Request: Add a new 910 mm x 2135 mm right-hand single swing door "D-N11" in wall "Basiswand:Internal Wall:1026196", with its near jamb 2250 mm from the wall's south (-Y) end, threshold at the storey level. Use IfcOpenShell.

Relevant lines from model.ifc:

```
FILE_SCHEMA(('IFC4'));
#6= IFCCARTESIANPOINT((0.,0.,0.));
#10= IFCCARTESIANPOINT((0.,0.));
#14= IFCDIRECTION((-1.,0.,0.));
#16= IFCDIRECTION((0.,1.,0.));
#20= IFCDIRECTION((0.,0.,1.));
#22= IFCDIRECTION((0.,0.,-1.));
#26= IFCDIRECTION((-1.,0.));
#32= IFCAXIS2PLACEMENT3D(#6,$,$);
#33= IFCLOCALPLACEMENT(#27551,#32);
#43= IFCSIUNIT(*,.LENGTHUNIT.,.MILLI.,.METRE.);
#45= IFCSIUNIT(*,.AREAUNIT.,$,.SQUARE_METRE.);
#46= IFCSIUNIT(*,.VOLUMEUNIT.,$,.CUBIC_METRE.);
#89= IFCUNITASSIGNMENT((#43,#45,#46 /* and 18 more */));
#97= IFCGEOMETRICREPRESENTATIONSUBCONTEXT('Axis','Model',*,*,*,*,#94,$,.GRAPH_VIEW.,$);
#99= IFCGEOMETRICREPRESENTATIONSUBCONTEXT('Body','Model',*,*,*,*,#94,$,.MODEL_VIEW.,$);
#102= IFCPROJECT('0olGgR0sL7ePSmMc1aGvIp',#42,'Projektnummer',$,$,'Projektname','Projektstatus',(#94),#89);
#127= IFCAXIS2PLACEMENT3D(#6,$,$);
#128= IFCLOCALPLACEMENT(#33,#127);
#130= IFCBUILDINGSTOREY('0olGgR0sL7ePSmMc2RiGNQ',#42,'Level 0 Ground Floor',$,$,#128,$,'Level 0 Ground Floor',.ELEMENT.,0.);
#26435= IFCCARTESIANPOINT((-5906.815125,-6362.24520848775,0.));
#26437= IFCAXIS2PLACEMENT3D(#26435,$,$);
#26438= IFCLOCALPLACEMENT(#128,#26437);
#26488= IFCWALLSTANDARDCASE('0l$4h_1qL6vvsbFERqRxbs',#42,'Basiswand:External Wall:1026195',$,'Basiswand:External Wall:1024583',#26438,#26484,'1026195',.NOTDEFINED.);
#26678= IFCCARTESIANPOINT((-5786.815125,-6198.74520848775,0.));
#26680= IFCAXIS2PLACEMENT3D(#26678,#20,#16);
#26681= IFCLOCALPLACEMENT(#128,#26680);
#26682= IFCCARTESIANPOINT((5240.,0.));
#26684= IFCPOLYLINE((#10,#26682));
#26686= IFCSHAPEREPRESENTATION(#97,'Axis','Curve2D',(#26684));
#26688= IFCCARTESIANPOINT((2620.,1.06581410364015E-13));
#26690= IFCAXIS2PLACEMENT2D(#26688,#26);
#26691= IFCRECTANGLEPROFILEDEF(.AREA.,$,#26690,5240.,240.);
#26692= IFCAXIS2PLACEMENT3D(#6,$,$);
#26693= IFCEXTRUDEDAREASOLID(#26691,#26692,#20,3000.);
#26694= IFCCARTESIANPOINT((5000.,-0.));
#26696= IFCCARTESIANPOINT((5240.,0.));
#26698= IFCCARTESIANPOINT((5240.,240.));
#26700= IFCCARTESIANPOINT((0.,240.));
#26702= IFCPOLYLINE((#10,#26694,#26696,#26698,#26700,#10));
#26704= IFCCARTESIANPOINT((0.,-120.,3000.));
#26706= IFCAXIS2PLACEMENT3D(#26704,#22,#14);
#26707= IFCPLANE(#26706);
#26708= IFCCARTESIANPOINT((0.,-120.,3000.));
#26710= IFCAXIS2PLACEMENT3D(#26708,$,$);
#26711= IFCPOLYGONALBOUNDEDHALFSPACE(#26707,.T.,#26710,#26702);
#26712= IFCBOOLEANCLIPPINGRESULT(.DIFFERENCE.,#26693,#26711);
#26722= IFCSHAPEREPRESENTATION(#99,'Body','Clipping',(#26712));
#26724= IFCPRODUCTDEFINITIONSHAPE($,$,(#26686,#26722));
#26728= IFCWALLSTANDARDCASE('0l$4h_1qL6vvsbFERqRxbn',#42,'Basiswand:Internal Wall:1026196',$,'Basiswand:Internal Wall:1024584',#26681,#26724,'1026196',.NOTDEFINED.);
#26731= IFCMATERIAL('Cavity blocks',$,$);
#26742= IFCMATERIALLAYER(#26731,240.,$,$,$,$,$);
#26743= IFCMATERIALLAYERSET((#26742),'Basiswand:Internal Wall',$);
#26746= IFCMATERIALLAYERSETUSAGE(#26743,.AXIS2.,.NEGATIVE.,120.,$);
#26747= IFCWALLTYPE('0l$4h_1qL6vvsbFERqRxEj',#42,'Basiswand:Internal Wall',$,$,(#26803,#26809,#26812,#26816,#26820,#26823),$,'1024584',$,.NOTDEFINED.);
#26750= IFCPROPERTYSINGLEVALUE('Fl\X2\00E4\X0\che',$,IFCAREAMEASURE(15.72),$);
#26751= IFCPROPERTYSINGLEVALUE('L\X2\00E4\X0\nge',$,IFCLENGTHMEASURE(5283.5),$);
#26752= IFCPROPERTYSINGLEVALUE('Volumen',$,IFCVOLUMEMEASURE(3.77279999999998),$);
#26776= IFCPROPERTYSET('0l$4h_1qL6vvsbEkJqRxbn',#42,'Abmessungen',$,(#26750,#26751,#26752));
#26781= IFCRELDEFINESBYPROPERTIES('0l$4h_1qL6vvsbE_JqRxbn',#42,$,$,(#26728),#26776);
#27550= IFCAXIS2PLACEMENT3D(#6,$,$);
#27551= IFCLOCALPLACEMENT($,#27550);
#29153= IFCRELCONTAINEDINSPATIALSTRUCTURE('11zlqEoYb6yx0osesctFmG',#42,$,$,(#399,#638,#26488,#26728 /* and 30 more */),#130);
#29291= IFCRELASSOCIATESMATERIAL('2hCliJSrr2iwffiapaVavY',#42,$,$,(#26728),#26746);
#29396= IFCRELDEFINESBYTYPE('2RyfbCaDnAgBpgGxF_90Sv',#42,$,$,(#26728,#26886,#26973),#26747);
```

```python
import numpy as np
import ifcopenshell
import ifcopenshell.api.feature
import ifcopenshell.api.geometry
import ifcopenshell.api.pset
import ifcopenshell.api.root
import ifcopenshell.api.spatial
import ifcopenshell.geom
import ifcopenshell.util.element
import ifcopenshell.util.placement
import ifcopenshell.util.representation
import ifcopenshell.util.shape
import ifcopenshell.util.unit

model = ifcopenshell.open("model.ifc")
unit_scale = ifcopenshell.util.unit.calculate_unit_scale(model)
area_scale = ifcopenshell.util.unit.calculate_unit_scale(model, "AREAUNIT")
volume_scale = ifcopenshell.util.unit.calculate_unit_scale(model, "VOLUMEUNIT")
settings = ifcopenshell.geom.settings()


def volume(element):
    """Net volume in cubic metres, openings subtracted."""
    shape = ifcopenshell.geom.create_shape(settings, element)
    return ifcopenshell.util.shape.get_volume(shape.geometry)


wall = model.by_id(26728)
storey = ifcopenshell.util.element.get_container(wall, ifc_class="IfcBuildingStorey")
context = ifcopenshell.util.representation.get_context(model, "Model", "Body", "MODEL_VIEW")
before = volume(wall)

width, height, from_end, sill = 0.91, 2.135, 2.25, 0.0  # metres

# The wall runs along its own X axis, and the end named is its -X end.
wall_shape = ifcopenshell.geom.create_shape(settings, wall)
x, y, z = ifcopenshell.util.shape.get_vertices(wall_shape.geometry).T
start = x.min() + from_end
face, thickness = float(y.min()), float(y.max() - y.min())
wall_matrix = ifcopenshell.util.placement.get_local_placement(wall.ObjectPlacement)
level = ifcopenshell.util.placement.get_local_placement(storey.ObjectPlacement)[2, 3]


def in_wall(x, y):
    """Placement at x, y metres in the wall's axes, at sill height."""
    matrix = wall_matrix.copy()
    matrix[:, 3] = wall_matrix @ np.array([x / unit_scale, y / unit_scale, 0.0, 1.0])
    matrix[2, 3] = level + sill / unit_scale
    return matrix


# Opening: a box that overshoots both wall faces by 50 mm.
opening = ifcopenshell.api.root.create_entity(model, ifc_class="IfcOpeningElement", predefined_type="OPENING")
box = ifcopenshell.api.geometry.add_wall_representation(
    model, context=context, length=width, height=height, thickness=thickness + 0.1
)
ifcopenshell.api.geometry.assign_representation(model, product=opening, representation=box)
ifcopenshell.api.geometry.edit_object_placement(model, product=opening, matrix=in_wall(start, face - 0.05), is_si=False)
ifcopenshell.api.feature.add_feature(model, feature=opening, element=wall)

door = ifcopenshell.api.root.create_entity(model, ifc_class="IfcDoor", name="D-N11", predefined_type="DOOR")
door.OverallWidth, door.OverallHeight = width / unit_scale, height / unit_scale
door.OperationType = "SINGLE_SWING_RIGHT"
body = ifcopenshell.api.geometry.add_door_representation(
    model,
    context=context,
    overall_width=door.OverallWidth,
    overall_height=door.OverallHeight,
    operation_type="SINGLE_SWING_RIGHT",
    lining_properties={"LiningDepth": thickness / unit_scale, "ThresholdDepth": thickness / unit_scale},
)
ifcopenshell.api.geometry.assign_representation(model, product=door, representation=body)
ifcopenshell.api.spatial.assign_container(model, products=[door], relating_structure=storey)
ifcopenshell.api.feature.add_filling(model, opening=opening, element=door)

# The lining spans the wall, so the door starts at the wall face.
ifcopenshell.api.geometry.edit_object_placement(model, product=door, matrix=in_wall(start, face), is_si=False)

after = volume(wall)

# Update the wall's stored quantities.
pset = model.by_id(ifcopenshell.util.element.get_pset(wall, "Abmessungen", should_inherit=False)["id"])
ifcopenshell.api.pset.edit_pset(model, pset=pset, properties={
    "Fläche": model.create_entity("IfcAreaMeasure", after / thickness / area_scale),
    "Volumen": model.create_entity("IfcVolumeMeasure", after / volume_scale),
})

print(f"wall volume {before:.3f} -> {after:.3f} m3")

model.write("model_updated.ifc")
```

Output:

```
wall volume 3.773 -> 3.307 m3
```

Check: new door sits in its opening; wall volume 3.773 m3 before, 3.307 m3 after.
